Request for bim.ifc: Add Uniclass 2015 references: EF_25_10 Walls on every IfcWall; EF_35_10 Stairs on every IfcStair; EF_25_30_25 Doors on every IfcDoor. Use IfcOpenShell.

First a look at what the model holds.

```python
import ifcopenshell

model = ifcopenshell.open("bim.ifc")
print(model.schema)
print("classifications:", [c.Name for c in model.by_type("IfcClassification")])
for ifc_class in ("IfcDoor", "IfcRoof", "IfcStair", "IfcWall", "IfcWindow"):
    print(ifc_class, len(model.by_type(ifc_class)))
```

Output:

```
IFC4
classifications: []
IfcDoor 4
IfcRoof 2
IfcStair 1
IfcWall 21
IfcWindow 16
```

```python
import ifcopenshell
import ifcopenshell.api.classification

model = ifcopenshell.open("bim.ifc")

system = ifcopenshell.api.classification.add_classification(model, classification="Uniclass 2015")

codes = {
    "IfcWall": ("EF_25_10", "Walls"),
    "IfcStair": ("EF_35_10", "Stairs"),
    "IfcDoor": ("EF_25_30_25", "Doors"),
}
for ifc_class, (code, name) in codes.items():
    products = model.by_type(ifc_class)
    ifcopenshell.api.classification.add_reference(
        model, products=products, classification=system, identification=code, name=name
    )
    print(code, len(products))

model.write("bim_updated.ifc")
```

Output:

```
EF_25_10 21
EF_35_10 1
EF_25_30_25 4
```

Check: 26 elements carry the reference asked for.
